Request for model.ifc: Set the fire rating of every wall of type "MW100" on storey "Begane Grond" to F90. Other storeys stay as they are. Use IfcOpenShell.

First a look at what the model holds.

```python
import ifcopenshell
import ifcopenshell.util.element

model = ifcopenshell.open("model.ifc")
print(model.schema)
storey = next(s for s in model.by_type("IfcBuildingStorey") if s.Name == "Begane Grond")
walls = [e for e in ifcopenshell.util.element.get_decomposition(storey) if e.is_a("IfcWall")]
seen = {}
for e in walls:
    element_type = ifcopenshell.util.element.get_type(e)
    key = (element_type.Name if element_type != e and element_type else None, ifcopenshell.util.element.get_pset(e, "Pset_WallCommon", "FireRating"))
    seen[key] = seen.get(key, 0) + 1
for (name, value), count in sorted(seen.items(), key=str):
    print(count, "x", name, "|", value)
```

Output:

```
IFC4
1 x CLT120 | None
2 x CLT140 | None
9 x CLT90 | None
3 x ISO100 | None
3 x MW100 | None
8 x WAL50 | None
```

```python
import ifcopenshell
import ifcopenshell.api.pset
import ifcopenshell.util.element

model = ifcopenshell.open("model.ifc")

storey = next(s for s in model.by_type("IfcBuildingStorey") if s.Name == "Begane Grond")
walls = [e for e in ifcopenshell.util.element.get_decomposition(storey) if e.is_a("IfcWall")]

count = 0
for e in walls:
    element_type = ifcopenshell.util.element.get_type(e)
    if element_type in (None, e) or element_type.Name != "MW100":
        continue
    # add_pset returns the element's existing set when there is one.
    pset = ifcopenshell.api.pset.add_pset(model, product=e, name="Pset_WallCommon")
    ifcopenshell.api.pset.edit_pset(model, pset=pset, properties={"FireRating": "F90"})
    count += 1

print(count, "walls updated")

model.write("model_v2.ifc")
```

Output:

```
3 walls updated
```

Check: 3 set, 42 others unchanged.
